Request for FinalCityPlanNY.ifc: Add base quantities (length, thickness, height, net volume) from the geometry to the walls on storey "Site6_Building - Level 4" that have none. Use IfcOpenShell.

First a look at what the model holds.

```python
import ifcopenshell
import ifcopenshell.util.element
import ifcopenshell.util.unit

model = ifcopenshell.open("FinalCityPlanNY.ifc")
print(model.schema)
for unit_type in ("LENGTHUNIT", "AREAUNIT", "VOLUMEUNIT"):
    print(unit_type, ifcopenshell.util.unit.calculate_unit_scale(model, unit_type))
storey = next(s for s in model.by_type("IfcBuildingStorey") if s.Name == "Site6_Building - Level 4")
walls = [e for e in ifcopenshell.util.element.get_decomposition(storey) if e.is_a("IfcWall")]
for e in sorted(walls, key=lambda e: e.id()):
    print(e.id(), e.is_a(), e.Name, list(ifcopenshell.util.element.get_psets(e, qtos_only=True)), sep=" | ")
```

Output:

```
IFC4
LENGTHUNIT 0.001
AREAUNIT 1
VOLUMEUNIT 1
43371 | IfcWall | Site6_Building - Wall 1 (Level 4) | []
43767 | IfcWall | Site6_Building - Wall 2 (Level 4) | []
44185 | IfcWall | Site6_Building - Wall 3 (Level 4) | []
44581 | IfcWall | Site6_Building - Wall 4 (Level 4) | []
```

```python
import ifcopenshell
import ifcopenshell.api.pset
import ifcopenshell.geom
import ifcopenshell.util.element
import ifcopenshell.util.shape
import ifcopenshell.util.unit

model = ifcopenshell.open("FinalCityPlanNY.ifc")
unit_scale = ifcopenshell.util.unit.calculate_unit_scale(model)
volume_scale = ifcopenshell.util.unit.calculate_unit_scale(model, "VOLUMEUNIT")
settings = ifcopenshell.geom.settings()

storey = next(s for s in model.by_type("IfcBuildingStorey") if s.Name == "Site6_Building - Level 4")
walls = [e for e in ifcopenshell.util.element.get_decomposition(storey) if e.is_a("IfcWall")]

for e in sorted(walls, key=lambda e: e.id()):
    if ifcopenshell.util.element.get_psets(e, qtos_only=True, should_inherit=False):
        continue
    # Geometry comes back in metres, in the element's own axes.
    shape = ifcopenshell.geom.create_shape(settings, e)
    values = {
        "Length": ifcopenshell.util.shape.get_x(shape.geometry) / unit_scale,
        "Width": ifcopenshell.util.shape.get_y(shape.geometry) / unit_scale,
        "Height": ifcopenshell.util.shape.get_z(shape.geometry) / unit_scale,
        "NetVolume": ifcopenshell.util.shape.get_volume(shape.geometry) / volume_scale,
    }
    qto = ifcopenshell.api.pset.add_qto(model, product=e, name="Qto_WallBaseQuantities")
    ifcopenshell.api.pset.edit_qto(model, qto=qto, properties=values)
    print(e.id(), {k: round(v, 3) for k, v in values.items()})

model.write("FinalCityPlanNY_rev.ifc")
```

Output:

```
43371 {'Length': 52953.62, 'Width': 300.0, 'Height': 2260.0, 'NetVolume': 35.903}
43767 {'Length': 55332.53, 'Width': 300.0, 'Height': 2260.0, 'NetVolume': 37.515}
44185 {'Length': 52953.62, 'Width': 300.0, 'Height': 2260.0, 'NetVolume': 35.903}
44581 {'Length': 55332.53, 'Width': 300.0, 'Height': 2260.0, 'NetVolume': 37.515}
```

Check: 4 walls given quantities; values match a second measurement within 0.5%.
